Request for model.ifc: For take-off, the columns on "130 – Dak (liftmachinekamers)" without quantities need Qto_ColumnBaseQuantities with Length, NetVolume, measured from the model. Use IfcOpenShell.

First a look at what the model holds.

```python
import ifcopenshell
import ifcopenshell.util.element
import ifcopenshell.util.unit

model = ifcopenshell.open("model.ifc")
print(model.schema)
for unit_type in ("LENGTHUNIT", "AREAUNIT", "VOLUMEUNIT"):
    print(unit_type, ifcopenshell.util.unit.calculate_unit_scale(model, unit_type))
storey = next(s for s in model.by_type("IfcBuildingStorey") if s.Name == "130 – Dak (liftmachinekamers)")
columns = [e for e in ifcopenshell.util.element.get_decomposition(storey) if e.is_a("IfcColumn")]
for e in sorted(columns, key=lambda e: e.id()):
    print(e.id(), e.is_a(), e.Name, list(ifcopenshell.util.element.get_psets(e, qtos_only=True)), sep=" | ")
```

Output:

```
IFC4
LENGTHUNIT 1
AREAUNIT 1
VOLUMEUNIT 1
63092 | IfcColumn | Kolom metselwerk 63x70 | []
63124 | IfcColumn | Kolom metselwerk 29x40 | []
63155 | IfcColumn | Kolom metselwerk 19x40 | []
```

```python
import ifcopenshell
import ifcopenshell.api.pset
import ifcopenshell.geom
import ifcopenshell.util.element
import ifcopenshell.util.shape
import ifcopenshell.util.unit

model = ifcopenshell.open("model.ifc")
unit_scale = ifcopenshell.util.unit.calculate_unit_scale(model)
volume_scale = ifcopenshell.util.unit.calculate_unit_scale(model, "VOLUMEUNIT")
settings = ifcopenshell.geom.settings()

storey = next(s for s in model.by_type("IfcBuildingStorey") if s.Name == "130 – Dak (liftmachinekamers)")
columns = [e for e in ifcopenshell.util.element.get_decomposition(storey) if e.is_a("IfcColumn")]

for e in sorted(columns, key=lambda e: e.id()):
    if ifcopenshell.util.element.get_psets(e, qtos_only=True, should_inherit=False):
        continue
    # Geometry comes back in metres, in the element's own axes.
    shape = ifcopenshell.geom.create_shape(settings, e)
    values = {
        "Length": ifcopenshell.util.shape.get_z(shape.geometry) / unit_scale,
        "NetVolume": ifcopenshell.util.shape.get_volume(shape.geometry) / volume_scale,
    }
    qto = ifcopenshell.api.pset.add_qto(model, product=e, name="Qto_ColumnBaseQuantities")
    ifcopenshell.api.pset.edit_qto(model, qto=qto, properties=values)
    print(e.id(), {k: round(v, 3) for k, v in values.items()})

model.write("model_v2.ifc")
```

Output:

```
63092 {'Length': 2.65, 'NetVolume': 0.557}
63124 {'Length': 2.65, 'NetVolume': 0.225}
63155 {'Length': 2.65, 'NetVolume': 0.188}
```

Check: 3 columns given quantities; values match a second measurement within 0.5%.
